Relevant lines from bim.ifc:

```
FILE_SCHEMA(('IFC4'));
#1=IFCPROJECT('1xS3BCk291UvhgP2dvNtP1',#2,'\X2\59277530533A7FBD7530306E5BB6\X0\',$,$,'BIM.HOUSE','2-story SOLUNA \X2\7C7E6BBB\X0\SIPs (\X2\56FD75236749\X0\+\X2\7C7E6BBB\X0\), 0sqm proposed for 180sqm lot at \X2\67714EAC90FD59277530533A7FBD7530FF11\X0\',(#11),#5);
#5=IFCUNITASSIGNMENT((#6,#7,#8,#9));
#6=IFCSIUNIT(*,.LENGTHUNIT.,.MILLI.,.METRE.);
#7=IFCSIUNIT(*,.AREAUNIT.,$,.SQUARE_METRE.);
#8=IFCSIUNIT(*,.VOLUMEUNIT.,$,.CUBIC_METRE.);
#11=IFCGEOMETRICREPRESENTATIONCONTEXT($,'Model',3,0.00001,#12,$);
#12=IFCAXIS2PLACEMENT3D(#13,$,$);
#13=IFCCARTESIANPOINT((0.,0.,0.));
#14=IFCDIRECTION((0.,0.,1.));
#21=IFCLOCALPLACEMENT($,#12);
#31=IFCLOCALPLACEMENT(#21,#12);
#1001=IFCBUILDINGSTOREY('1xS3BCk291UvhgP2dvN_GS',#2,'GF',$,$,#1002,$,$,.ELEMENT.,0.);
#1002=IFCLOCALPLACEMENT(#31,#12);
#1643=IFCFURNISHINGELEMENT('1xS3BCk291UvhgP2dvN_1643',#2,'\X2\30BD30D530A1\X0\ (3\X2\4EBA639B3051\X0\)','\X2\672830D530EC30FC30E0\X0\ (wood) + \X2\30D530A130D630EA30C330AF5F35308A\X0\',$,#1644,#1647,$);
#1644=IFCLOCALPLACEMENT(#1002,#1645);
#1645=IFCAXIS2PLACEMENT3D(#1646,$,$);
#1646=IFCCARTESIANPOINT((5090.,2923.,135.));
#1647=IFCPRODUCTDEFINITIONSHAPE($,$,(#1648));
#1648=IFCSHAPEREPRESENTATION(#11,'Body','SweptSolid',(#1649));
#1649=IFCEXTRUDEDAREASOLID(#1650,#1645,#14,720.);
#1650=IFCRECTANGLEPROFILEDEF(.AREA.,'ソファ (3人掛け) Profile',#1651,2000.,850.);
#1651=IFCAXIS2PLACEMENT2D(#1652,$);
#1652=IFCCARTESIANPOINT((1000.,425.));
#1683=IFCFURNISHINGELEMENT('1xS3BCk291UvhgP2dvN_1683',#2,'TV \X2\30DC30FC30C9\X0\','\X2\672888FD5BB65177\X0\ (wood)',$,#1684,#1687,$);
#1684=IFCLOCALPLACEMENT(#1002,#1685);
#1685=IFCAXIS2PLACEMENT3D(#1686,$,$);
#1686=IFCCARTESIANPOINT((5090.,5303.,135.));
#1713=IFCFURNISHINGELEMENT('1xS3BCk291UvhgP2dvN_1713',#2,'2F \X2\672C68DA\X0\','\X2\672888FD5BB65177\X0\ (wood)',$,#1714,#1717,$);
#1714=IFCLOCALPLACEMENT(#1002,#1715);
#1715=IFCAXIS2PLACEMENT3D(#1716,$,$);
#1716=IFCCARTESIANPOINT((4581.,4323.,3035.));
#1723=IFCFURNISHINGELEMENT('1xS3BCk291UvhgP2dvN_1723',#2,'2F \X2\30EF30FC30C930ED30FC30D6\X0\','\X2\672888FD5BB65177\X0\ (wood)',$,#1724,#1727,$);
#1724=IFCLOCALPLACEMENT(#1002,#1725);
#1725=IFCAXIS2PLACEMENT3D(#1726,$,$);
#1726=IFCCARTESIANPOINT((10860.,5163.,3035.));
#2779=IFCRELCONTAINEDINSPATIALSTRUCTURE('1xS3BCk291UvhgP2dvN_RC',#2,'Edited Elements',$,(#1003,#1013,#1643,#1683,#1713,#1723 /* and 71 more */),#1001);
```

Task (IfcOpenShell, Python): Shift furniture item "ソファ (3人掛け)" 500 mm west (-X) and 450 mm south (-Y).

```python
import ifcopenshell
import ifcopenshell.api.geometry
import ifcopenshell.util.placement
import ifcopenshell.util.unit

model = ifcopenshell.open("bim.ifc")
unit_scale = ifcopenshell.util.unit.calculate_unit_scale(model)

item = model.by_guid("1xS3BCk291UvhgP2dvN_1643")
matrix = ifcopenshell.util.placement.get_local_placement(item.ObjectPlacement)
matrix[0, 3] -= 0.5 / unit_scale
matrix[1, 3] -= 0.45 / unit_scale
ifcopenshell.api.geometry.edit_object_placement(model, product=item, matrix=matrix, is_si=False)

print(ifcopenshell.util.placement.get_local_placement(item.ObjectPlacement).round(3) + 0.0)

model.write("bim_updated.ifc")
```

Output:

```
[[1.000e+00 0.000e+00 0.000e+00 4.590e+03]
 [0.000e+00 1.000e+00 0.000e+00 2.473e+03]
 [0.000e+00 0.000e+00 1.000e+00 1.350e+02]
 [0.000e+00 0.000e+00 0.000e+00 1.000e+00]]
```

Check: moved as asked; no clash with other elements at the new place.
